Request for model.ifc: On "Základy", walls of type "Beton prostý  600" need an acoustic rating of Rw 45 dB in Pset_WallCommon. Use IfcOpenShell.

First a look at what the model holds.

```python
import ifcopenshell
import ifcopenshell.util.element

model = ifcopenshell.open("model.ifc")
print(model.schema)
storey = next(s for s in model.by_type("IfcBuildingStorey") if s.Name == "Základy")
walls = [e for e in ifcopenshell.util.element.get_decomposition(storey) if e.is_a("IfcWall")]
seen = {}
for e in walls:
    element_type = ifcopenshell.util.element.get_type(e)
    key = (element_type.Name if element_type != e and element_type else None, ifcopenshell.util.element.get_pset(e, "Pset_WallCommon", "AcousticRating"))
    seen[key] = seen.get(key, 0) + 1
for (name, value), count in sorted(seen.items(), key=str):
    print(count, "x", name, "|", value)
```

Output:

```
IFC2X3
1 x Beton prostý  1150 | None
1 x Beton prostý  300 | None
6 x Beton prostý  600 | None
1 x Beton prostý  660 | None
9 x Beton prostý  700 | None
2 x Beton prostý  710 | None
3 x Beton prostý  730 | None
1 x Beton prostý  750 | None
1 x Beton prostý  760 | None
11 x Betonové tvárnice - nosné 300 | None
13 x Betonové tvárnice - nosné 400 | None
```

```python
import ifcopenshell
import ifcopenshell.api.pset
import ifcopenshell.util.element

model = ifcopenshell.open("model.ifc")

storey = next(s for s in model.by_type("IfcBuildingStorey") if s.Name == "Základy")
walls = [e for e in ifcopenshell.util.element.get_decomposition(storey) if e.is_a("IfcWall")]

count = 0
for e in walls:
    element_type = ifcopenshell.util.element.get_type(e)
    if element_type in (None, e) or element_type.Name != "Beton prostý  600":
        continue
    # add_pset returns the element's existing set when there is one.
    pset = ifcopenshell.api.pset.add_pset(model, product=e, name="Pset_WallCommon")
    ifcopenshell.api.pset.edit_pset(model, pset=pset, properties={"AcousticRating": "Rw 45 dB"})
    count += 1

print(count, "walls updated")

model.write("model-out.ifc")
```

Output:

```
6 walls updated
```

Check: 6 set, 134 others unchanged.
